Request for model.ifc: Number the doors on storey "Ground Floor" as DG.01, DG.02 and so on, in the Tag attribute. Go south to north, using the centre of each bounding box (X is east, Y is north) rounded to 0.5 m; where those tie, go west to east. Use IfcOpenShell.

First a look at what the model holds.

```python
import ifcopenshell
import ifcopenshell.util.element
import ifcopenshell.util.placement

model = ifcopenshell.open("model.ifc")
print(model.schema)
storey = next(s for s in model.by_type("IfcBuildingStorey") if s.Name == "Ground Floor")
doors = [e for e in ifcopenshell.util.element.get_decomposition(storey) if e.is_a("IfcDoor")]
for e in sorted(doors, key=lambda e: e.id()):
    origin = ifcopenshell.util.placement.get_local_placement(e.ObjectPlacement)[:3, 3]
    print(e.id(), e.Tag, e.Name, origin.round(2) + 0.0, sep=" | ")
```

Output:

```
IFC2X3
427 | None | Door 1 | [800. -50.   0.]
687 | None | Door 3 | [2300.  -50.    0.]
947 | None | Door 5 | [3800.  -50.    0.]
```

```python
import ifcopenshell
import ifcopenshell.geom
import ifcopenshell.util.element
import ifcopenshell.util.shape

model = ifcopenshell.open("model.ifc")
settings = ifcopenshell.geom.settings()
settings.set("use-world-coords", True)


def centre(element):
    shape = ifcopenshell.geom.create_shape(settings, element)
    return ifcopenshell.util.shape.get_bbox_centroid(shape.geometry)


storey = next(s for s in model.by_type("IfcBuildingStorey") if s.Name == "Ground Floor")
doors = [e for e in ifcopenshell.util.element.get_decomposition(storey) if e.is_a("IfcDoor")]

# Insertion points can sit at a corner or the storey origin, so sort by the geometry (in metres).
centres = {e: centre(e) for e in doors}
doors.sort(key=lambda e: (round(centres[e][1] / 0.5), centres[e][0]))

for i, e in enumerate(doors, start=1):
    number = f"DG.{i:02d}"
    e.Tag = number
    print(e.id(), number)

model.write("model_v2.ifc")
```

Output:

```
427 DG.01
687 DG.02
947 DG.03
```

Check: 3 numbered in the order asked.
